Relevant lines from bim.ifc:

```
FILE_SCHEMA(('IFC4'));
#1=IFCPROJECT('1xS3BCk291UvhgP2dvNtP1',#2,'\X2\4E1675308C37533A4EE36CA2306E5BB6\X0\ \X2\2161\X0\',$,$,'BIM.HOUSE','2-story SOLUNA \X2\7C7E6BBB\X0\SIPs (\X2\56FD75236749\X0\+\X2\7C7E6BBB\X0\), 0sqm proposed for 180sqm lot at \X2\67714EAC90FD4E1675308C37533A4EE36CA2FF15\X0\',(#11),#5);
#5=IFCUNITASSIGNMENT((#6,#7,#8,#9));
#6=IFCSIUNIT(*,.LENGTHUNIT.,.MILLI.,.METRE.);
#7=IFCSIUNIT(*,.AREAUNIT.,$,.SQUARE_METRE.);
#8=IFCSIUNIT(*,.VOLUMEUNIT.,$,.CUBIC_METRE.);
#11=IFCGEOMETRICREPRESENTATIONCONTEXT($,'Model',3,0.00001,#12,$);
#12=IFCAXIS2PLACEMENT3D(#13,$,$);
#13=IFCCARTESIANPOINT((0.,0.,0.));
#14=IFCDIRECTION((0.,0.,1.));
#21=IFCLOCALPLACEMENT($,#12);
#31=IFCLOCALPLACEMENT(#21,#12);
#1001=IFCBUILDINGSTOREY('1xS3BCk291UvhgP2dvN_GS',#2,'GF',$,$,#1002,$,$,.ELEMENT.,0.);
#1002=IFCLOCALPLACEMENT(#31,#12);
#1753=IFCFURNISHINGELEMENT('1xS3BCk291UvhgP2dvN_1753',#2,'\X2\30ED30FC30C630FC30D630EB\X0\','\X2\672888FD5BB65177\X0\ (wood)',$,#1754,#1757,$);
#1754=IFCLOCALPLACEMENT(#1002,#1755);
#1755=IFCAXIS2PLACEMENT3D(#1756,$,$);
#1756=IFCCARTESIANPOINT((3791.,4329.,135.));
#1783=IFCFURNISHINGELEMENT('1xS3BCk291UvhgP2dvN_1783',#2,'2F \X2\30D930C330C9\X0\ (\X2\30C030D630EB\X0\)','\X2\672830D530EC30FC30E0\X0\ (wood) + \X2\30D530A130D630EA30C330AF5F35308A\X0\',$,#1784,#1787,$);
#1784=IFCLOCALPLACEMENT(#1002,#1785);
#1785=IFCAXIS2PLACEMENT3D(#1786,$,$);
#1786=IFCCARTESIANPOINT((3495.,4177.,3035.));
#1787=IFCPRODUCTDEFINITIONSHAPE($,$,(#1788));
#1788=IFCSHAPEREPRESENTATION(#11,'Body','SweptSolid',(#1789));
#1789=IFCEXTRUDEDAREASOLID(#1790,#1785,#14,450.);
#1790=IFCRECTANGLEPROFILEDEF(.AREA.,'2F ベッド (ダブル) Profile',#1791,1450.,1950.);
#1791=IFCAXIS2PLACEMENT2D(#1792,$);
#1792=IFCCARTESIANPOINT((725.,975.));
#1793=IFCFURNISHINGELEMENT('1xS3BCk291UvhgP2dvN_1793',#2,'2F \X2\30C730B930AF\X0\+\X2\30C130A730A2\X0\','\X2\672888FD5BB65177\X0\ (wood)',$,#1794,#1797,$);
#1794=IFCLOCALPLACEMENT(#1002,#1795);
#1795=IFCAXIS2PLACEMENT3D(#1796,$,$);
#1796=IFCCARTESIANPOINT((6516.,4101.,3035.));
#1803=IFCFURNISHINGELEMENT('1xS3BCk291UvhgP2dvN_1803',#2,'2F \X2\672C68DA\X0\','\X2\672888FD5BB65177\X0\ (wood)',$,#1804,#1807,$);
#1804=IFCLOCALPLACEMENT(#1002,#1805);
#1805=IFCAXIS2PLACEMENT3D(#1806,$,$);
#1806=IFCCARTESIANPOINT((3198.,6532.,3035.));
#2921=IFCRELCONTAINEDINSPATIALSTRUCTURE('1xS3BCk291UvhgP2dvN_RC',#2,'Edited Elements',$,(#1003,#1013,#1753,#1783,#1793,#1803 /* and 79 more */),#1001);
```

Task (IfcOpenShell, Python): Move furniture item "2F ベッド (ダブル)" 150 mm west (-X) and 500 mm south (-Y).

```python
import ifcopenshell
import ifcopenshell.api.geometry
import ifcopenshell.util.placement
import ifcopenshell.util.unit

model = ifcopenshell.open("bim.ifc")
unit_scale = ifcopenshell.util.unit.calculate_unit_scale(model)

item = model.by_guid("1xS3BCk291UvhgP2dvN_1783")
matrix = ifcopenshell.util.placement.get_local_placement(item.ObjectPlacement)
matrix[0, 3] -= 0.15 / unit_scale
matrix[1, 3] -= 0.5 / unit_scale
ifcopenshell.api.geometry.edit_object_placement(model, product=item, matrix=matrix, is_si=False)

print(ifcopenshell.util.placement.get_local_placement(item.ObjectPlacement).round(3) + 0.0)

model.write("bim_edited.ifc")
```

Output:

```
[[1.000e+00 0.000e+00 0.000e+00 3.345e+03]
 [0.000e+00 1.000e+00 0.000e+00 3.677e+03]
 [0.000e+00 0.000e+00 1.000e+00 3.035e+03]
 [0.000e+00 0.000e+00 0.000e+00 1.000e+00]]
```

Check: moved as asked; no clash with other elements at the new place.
